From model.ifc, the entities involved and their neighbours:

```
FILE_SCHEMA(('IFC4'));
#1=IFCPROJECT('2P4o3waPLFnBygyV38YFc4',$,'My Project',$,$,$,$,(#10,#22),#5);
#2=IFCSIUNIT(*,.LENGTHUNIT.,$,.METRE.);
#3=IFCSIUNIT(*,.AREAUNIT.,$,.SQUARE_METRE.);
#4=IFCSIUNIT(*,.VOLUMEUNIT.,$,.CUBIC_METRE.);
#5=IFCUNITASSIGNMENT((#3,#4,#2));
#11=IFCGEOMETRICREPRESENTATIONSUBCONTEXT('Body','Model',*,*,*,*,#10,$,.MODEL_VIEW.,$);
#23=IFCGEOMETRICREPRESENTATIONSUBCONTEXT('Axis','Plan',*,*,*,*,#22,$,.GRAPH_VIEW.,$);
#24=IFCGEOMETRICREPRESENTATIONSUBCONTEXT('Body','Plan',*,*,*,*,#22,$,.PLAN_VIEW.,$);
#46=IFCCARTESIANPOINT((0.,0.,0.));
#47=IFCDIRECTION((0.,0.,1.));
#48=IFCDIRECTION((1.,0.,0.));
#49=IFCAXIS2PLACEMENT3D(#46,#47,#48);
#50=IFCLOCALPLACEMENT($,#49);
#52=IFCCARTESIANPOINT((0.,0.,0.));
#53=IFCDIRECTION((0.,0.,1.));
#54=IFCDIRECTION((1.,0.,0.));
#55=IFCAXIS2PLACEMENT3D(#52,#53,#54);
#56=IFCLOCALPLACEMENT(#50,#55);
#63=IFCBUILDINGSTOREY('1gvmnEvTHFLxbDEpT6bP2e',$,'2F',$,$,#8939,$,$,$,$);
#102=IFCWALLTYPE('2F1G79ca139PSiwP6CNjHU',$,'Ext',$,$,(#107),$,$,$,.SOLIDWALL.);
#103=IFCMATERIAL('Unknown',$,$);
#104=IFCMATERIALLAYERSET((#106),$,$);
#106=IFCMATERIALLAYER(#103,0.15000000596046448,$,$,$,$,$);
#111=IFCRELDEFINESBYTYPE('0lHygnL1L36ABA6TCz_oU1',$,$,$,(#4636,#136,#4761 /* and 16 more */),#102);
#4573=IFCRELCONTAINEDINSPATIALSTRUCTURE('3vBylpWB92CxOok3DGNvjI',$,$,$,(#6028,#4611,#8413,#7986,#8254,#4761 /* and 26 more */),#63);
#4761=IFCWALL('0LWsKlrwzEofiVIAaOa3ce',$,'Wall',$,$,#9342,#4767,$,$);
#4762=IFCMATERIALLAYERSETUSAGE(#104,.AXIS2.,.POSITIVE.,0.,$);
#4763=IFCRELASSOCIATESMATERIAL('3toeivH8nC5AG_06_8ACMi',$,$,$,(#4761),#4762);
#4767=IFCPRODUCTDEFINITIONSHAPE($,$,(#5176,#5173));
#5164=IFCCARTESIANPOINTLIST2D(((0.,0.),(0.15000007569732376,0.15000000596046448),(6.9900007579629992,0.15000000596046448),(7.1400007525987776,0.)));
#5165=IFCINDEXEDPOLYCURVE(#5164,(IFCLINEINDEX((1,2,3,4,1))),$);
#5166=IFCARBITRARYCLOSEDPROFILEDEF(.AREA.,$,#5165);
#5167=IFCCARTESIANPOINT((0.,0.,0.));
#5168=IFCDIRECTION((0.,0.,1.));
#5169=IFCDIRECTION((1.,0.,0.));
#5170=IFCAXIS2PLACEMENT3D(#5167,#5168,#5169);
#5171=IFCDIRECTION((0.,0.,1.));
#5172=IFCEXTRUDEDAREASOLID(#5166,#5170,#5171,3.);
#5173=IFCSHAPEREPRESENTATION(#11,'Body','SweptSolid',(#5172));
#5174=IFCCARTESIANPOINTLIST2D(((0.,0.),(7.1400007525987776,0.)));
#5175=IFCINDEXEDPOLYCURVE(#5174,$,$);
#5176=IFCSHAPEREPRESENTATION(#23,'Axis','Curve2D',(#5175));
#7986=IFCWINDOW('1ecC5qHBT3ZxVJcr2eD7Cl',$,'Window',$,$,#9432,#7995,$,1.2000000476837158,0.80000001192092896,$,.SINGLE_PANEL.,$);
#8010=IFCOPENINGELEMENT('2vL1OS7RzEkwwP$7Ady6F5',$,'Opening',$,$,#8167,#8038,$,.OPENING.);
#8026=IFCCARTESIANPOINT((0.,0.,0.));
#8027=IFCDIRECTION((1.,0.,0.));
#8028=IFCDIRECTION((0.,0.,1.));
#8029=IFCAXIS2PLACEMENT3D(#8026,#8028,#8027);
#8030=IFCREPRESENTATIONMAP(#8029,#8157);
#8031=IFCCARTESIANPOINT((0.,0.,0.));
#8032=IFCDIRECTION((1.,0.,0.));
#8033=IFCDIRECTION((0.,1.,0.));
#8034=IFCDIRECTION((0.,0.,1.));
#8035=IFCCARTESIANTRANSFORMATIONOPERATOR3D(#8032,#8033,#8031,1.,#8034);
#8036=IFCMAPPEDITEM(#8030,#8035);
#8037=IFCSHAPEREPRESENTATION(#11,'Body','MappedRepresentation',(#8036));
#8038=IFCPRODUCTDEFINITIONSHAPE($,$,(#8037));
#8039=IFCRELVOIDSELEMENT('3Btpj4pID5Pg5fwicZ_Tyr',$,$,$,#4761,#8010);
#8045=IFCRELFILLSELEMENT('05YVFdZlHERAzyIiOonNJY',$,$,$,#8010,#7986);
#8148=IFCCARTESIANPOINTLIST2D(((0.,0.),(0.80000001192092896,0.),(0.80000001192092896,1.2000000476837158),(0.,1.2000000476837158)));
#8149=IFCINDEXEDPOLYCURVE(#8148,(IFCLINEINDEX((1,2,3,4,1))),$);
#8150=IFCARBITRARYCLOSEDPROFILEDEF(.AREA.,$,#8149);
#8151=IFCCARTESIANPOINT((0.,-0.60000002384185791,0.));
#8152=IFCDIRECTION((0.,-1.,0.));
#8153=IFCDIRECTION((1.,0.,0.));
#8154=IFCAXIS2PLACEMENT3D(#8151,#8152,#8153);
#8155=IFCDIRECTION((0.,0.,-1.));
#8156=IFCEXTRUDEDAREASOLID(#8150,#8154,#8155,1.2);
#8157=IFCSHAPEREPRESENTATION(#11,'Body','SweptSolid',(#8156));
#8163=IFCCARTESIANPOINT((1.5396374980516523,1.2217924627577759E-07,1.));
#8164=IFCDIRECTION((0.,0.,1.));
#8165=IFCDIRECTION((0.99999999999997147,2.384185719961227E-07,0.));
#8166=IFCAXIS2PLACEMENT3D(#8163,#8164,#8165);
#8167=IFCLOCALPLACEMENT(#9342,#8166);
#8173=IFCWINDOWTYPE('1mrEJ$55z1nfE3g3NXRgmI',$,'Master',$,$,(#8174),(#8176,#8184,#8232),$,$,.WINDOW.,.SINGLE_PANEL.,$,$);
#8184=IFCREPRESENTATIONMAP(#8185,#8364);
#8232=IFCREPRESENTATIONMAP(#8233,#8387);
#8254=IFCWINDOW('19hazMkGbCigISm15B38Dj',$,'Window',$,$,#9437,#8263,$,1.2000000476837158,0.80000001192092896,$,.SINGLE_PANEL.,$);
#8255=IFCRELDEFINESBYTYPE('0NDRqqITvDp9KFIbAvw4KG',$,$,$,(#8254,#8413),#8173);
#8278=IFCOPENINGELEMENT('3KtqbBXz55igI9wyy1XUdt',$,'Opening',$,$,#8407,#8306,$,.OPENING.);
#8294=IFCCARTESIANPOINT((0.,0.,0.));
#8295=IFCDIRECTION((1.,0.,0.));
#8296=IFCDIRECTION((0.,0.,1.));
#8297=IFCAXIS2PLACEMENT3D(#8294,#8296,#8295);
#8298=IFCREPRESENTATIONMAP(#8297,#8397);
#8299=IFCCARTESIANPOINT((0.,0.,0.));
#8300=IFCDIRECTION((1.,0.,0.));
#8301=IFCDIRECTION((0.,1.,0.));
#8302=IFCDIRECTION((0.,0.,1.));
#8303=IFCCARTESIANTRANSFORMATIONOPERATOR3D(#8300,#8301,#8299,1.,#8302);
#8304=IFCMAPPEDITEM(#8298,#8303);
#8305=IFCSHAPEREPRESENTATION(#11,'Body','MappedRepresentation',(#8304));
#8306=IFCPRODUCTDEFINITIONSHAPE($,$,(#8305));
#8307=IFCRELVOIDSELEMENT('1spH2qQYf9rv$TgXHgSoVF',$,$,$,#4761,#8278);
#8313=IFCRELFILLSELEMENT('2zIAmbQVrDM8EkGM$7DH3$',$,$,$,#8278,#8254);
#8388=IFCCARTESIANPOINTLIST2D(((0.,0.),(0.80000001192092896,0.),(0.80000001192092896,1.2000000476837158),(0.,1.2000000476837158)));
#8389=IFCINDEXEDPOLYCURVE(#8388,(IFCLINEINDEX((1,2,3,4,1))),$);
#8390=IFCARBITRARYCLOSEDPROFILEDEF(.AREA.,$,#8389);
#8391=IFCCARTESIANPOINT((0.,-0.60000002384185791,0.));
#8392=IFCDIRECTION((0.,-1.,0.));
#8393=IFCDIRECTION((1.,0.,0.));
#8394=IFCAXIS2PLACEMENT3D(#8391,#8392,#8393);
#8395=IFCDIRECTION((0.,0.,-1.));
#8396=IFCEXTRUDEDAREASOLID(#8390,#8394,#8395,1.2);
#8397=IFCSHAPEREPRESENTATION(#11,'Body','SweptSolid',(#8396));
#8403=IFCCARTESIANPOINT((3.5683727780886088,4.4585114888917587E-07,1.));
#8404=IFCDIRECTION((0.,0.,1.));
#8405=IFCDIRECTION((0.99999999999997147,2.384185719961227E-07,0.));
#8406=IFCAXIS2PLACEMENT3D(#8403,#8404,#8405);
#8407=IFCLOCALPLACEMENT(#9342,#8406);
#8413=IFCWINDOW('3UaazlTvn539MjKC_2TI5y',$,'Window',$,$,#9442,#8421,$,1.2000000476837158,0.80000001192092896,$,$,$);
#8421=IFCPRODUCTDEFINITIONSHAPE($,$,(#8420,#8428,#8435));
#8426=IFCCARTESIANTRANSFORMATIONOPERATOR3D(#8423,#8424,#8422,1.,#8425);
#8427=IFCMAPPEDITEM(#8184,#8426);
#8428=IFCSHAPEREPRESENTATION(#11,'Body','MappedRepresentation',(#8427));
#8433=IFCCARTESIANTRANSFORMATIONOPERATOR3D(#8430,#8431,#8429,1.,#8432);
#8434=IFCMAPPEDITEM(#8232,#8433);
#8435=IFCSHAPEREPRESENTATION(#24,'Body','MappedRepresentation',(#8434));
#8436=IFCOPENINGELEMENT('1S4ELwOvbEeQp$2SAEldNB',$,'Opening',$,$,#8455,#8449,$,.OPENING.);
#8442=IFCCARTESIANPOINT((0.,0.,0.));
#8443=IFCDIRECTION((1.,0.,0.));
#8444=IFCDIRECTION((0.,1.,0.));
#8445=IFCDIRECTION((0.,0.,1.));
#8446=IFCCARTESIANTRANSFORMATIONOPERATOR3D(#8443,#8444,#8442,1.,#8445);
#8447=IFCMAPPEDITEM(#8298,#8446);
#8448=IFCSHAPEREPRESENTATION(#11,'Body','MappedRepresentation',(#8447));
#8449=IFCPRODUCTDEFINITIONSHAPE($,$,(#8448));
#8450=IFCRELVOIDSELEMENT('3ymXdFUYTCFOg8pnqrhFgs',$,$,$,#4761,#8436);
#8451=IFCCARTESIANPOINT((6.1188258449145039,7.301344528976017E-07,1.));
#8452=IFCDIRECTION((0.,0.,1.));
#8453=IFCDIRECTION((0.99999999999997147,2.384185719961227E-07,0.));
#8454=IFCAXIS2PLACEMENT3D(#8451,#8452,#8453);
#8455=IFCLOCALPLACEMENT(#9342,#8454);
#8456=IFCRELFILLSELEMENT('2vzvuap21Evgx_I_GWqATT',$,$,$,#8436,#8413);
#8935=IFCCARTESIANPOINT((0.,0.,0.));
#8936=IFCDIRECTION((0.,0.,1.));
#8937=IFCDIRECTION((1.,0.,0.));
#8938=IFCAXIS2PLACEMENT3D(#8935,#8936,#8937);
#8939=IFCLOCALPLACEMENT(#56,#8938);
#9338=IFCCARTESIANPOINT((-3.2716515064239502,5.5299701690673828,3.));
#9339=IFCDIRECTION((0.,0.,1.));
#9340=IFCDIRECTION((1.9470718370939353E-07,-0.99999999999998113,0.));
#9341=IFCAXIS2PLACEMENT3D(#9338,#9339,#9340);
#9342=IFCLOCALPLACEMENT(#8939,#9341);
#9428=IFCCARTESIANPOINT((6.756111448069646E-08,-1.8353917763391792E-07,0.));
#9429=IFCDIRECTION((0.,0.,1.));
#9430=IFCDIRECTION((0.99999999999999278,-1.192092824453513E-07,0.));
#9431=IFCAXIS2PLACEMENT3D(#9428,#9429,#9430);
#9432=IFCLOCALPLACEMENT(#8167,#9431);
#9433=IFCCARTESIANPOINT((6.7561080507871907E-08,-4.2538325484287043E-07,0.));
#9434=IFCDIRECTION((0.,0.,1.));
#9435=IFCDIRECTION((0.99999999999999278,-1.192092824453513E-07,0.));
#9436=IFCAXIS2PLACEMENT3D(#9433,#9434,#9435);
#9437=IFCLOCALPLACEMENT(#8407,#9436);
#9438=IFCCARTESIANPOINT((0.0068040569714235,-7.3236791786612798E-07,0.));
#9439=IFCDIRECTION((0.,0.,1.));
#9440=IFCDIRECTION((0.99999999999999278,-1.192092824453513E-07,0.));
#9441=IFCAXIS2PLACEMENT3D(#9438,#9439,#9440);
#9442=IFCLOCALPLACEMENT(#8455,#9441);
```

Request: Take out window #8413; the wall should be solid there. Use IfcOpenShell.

```python
import ifcopenshell
import ifcopenshell.api.feature
import ifcopenshell.api.root
import ifcopenshell.geom
import ifcopenshell.util.shape

model = ifcopenshell.open("model.ifc")
settings = ifcopenshell.geom.settings()


def volume(element):
    """Net volume in cubic metres, openings subtracted."""
    shape = ifcopenshell.geom.create_shape(settings, element)
    return ifcopenshell.util.shape.get_volume(shape.geometry)


window = model.by_guid("3UaazlTvn539MjKC_2TI5y")
opening = window.FillsVoids[0].RelatingOpeningElement
wall = opening.VoidsElements[0].RelatingBuildingElement
before = volume(wall)

ifcopenshell.api.root.remove_product(model, product=window)
ifcopenshell.api.feature.remove_feature(model, feature=opening)

after = volume(wall)

print(f"wall volume {before:.3f} -> {after:.3f} m3")

model.write("model_v2.ifc")
```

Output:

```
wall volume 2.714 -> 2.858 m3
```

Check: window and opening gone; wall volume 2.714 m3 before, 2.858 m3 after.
